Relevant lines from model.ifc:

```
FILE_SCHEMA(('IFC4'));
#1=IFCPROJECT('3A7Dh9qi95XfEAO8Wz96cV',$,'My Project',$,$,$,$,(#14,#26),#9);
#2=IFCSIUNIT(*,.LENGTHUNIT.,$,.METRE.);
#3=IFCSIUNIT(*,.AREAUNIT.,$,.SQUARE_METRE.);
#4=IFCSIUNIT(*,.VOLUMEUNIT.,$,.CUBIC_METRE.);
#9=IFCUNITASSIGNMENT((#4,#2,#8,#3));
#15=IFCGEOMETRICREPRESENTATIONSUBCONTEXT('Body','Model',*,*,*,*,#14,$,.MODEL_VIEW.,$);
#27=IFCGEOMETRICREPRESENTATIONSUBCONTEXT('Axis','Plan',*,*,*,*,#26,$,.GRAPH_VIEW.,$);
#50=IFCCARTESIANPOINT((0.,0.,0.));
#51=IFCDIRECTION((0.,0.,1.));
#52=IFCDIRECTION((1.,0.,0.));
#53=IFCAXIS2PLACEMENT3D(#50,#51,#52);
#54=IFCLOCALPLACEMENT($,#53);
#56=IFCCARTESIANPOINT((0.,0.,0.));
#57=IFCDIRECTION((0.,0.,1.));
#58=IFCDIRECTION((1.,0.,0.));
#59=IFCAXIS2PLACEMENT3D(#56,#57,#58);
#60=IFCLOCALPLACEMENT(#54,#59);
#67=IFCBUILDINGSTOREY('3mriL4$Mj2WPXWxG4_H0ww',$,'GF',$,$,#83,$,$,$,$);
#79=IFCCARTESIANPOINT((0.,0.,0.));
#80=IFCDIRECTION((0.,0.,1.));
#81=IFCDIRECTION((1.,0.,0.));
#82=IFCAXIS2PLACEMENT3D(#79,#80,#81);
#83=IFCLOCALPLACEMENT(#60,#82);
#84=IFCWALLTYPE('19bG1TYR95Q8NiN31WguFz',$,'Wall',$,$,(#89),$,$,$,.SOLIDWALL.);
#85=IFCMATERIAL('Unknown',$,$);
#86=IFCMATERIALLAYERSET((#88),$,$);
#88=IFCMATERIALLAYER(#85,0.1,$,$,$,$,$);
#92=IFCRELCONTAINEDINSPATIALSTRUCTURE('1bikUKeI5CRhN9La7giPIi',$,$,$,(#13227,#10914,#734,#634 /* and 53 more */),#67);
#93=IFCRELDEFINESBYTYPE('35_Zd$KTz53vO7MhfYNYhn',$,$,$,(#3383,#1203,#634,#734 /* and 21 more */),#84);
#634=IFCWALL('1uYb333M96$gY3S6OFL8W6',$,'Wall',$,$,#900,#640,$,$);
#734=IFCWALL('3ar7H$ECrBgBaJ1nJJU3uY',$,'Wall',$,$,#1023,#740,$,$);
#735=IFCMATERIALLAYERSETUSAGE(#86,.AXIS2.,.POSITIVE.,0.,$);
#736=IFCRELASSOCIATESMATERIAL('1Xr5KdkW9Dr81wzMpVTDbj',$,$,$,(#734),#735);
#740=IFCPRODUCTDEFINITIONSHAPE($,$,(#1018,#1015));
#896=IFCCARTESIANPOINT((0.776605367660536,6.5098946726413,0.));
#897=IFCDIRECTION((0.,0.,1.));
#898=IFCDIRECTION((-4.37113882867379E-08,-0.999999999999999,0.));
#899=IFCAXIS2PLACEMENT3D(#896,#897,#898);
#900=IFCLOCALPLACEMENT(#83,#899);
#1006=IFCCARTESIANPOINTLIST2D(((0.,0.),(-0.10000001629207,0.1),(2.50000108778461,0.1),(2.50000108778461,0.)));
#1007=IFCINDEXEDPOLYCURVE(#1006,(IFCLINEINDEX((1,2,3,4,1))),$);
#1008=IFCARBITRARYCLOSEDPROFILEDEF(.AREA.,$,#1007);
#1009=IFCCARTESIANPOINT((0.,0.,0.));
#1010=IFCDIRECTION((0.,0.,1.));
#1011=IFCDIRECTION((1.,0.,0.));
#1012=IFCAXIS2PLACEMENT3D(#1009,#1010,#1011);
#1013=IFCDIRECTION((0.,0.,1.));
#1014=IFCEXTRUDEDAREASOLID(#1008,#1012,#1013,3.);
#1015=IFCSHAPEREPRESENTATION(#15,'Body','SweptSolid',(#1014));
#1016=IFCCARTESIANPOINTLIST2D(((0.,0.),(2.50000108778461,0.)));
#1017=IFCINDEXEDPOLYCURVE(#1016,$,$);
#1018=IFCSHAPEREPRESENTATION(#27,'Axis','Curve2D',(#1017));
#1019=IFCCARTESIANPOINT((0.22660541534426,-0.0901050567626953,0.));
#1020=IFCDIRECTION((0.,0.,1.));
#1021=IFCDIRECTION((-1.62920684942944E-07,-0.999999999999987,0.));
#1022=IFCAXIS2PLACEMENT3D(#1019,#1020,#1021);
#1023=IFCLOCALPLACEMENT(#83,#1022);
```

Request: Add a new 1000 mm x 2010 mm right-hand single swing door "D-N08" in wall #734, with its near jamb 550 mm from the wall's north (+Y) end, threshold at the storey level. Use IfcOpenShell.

```python
import numpy as np
import ifcopenshell
import ifcopenshell.api.feature
import ifcopenshell.api.geometry
import ifcopenshell.api.root
import ifcopenshell.api.spatial
import ifcopenshell.geom
import ifcopenshell.util.element
import ifcopenshell.util.placement
import ifcopenshell.util.representation
import ifcopenshell.util.shape
import ifcopenshell.util.unit

model = ifcopenshell.open("model.ifc")
unit_scale = ifcopenshell.util.unit.calculate_unit_scale(model)
settings = ifcopenshell.geom.settings()


def volume(element):
    """Net volume in cubic metres, openings subtracted."""
    shape = ifcopenshell.geom.create_shape(settings, element)
    return ifcopenshell.util.shape.get_volume(shape.geometry)


wall = model.by_guid("3ar7H$ECrBgBaJ1nJJU3uY")
storey = ifcopenshell.util.element.get_container(wall, ifc_class="IfcBuildingStorey")
context = ifcopenshell.util.representation.get_context(model, "Model", "Body", "MODEL_VIEW")
before = volume(wall)

width, height, from_end, sill = 1, 2.01, 0.55, 0.0  # metres

# The wall runs along its own X axis, and the end named is its -X end.
wall_shape = ifcopenshell.geom.create_shape(settings, wall)
x, y, z = ifcopenshell.util.shape.get_vertices(wall_shape.geometry).T
start = x.min() + from_end
face, thickness = float(y.min()), float(y.max() - y.min())
wall_matrix = ifcopenshell.util.placement.get_local_placement(wall.ObjectPlacement)
level = ifcopenshell.util.placement.get_local_placement(storey.ObjectPlacement)[2, 3]


def in_wall(x, y):
    """Placement at x, y metres in the wall's axes, at sill height."""
    matrix = wall_matrix.copy()
    matrix[:, 3] = wall_matrix @ np.array([x / unit_scale, y / unit_scale, 0.0, 1.0])
    matrix[2, 3] = level + sill / unit_scale
    return matrix


# Opening: a box that overshoots both wall faces by 50 mm.
opening = ifcopenshell.api.root.create_entity(model, ifc_class="IfcOpeningElement", predefined_type="OPENING")
box = ifcopenshell.api.geometry.add_wall_representation(
    model, context=context, length=width, height=height, thickness=thickness + 0.1
)
ifcopenshell.api.geometry.assign_representation(model, product=opening, representation=box)
ifcopenshell.api.geometry.edit_object_placement(model, product=opening, matrix=in_wall(start, face - 0.05), is_si=False)
ifcopenshell.api.feature.add_feature(model, feature=opening, element=wall)

door = ifcopenshell.api.root.create_entity(model, ifc_class="IfcDoor", name="D-N08", predefined_type="DOOR")
door.OverallWidth, door.OverallHeight = width / unit_scale, height / unit_scale
door.OperationType = "SINGLE_SWING_RIGHT"
body = ifcopenshell.api.geometry.add_door_representation(
    model,
    context=context,
    overall_width=door.OverallWidth,
    overall_height=door.OverallHeight,
    operation_type="SINGLE_SWING_RIGHT",
    lining_properties={"LiningDepth": thickness / unit_scale, "ThresholdDepth": thickness / unit_scale},
)
ifcopenshell.api.geometry.assign_representation(model, product=door, representation=body)
ifcopenshell.api.spatial.assign_container(model, products=[door], relating_structure=storey)
ifcopenshell.api.feature.add_filling(model, opening=opening, element=door)

# The lining spans the wall, so the door starts at the wall face.
ifcopenshell.api.geometry.edit_object_placement(model, product=door, matrix=in_wall(start, face), is_si=False)

after = volume(wall)

print(f"wall volume {before:.3f} -> {after:.3f} m3")

model.write("model_rev.ifc")
```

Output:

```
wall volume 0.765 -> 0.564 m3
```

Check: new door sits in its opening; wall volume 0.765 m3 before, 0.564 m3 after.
